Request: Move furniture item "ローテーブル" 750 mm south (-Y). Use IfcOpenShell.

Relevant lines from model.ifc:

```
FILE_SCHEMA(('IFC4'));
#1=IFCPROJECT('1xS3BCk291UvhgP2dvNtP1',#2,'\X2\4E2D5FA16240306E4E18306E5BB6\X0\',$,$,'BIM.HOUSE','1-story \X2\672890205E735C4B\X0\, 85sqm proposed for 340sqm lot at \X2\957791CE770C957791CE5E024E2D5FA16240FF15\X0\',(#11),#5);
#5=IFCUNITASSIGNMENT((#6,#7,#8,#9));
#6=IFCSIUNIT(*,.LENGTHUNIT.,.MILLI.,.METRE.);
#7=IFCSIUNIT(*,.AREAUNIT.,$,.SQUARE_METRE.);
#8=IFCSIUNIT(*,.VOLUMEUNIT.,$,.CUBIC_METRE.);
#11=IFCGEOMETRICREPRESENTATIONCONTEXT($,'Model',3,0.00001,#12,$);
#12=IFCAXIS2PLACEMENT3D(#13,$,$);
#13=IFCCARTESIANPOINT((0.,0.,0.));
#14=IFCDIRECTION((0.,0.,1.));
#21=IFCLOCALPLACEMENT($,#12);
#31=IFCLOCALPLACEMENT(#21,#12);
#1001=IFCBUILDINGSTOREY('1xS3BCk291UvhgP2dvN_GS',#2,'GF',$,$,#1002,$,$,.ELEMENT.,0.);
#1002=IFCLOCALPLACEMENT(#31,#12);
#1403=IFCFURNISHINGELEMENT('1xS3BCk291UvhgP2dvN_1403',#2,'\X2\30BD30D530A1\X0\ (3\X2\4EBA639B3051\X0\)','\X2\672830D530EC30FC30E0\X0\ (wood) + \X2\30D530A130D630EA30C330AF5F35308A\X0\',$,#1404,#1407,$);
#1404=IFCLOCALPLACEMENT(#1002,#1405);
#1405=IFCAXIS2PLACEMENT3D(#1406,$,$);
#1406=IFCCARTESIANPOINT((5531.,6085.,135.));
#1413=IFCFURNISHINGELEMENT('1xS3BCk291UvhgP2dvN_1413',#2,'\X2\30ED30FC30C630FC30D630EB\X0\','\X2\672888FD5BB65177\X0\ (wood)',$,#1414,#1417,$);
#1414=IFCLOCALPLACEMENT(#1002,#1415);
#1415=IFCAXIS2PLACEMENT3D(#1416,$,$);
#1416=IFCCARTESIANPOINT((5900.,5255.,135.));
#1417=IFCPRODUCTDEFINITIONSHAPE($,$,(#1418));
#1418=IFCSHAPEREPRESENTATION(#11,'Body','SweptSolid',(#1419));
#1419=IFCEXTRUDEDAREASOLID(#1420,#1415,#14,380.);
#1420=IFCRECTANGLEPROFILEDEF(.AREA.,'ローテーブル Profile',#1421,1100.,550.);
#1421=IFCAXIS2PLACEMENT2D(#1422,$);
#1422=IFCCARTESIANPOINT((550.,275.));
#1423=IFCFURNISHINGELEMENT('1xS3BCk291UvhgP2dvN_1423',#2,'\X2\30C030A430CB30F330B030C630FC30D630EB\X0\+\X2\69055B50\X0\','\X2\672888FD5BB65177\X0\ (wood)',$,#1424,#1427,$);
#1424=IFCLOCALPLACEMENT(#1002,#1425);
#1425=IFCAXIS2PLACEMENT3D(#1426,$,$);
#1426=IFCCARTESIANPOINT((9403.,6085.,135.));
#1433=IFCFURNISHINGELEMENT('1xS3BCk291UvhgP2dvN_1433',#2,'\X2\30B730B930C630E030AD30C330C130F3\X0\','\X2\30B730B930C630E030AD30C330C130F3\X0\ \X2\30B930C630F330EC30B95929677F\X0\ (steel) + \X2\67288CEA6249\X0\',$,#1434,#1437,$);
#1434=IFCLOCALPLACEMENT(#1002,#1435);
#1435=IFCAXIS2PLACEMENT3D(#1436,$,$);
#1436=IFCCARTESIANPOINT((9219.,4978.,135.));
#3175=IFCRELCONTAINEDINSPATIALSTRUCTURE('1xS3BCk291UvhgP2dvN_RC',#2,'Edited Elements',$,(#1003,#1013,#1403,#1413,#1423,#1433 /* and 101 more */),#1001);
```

```python
import ifcopenshell
import ifcopenshell.api.geometry
import ifcopenshell.util.placement
import ifcopenshell.util.unit

model = ifcopenshell.open("model.ifc")
unit_scale = ifcopenshell.util.unit.calculate_unit_scale(model)

item = model.by_guid("1xS3BCk291UvhgP2dvN_1413")
matrix = ifcopenshell.util.placement.get_local_placement(item.ObjectPlacement)
matrix[1, 3] -= 0.75 / unit_scale
ifcopenshell.api.geometry.edit_object_placement(model, product=item, matrix=matrix, is_si=False)

print(ifcopenshell.util.placement.get_local_placement(item.ObjectPlacement).round(3) + 0.0)

model.write("model_v2.ifc")
```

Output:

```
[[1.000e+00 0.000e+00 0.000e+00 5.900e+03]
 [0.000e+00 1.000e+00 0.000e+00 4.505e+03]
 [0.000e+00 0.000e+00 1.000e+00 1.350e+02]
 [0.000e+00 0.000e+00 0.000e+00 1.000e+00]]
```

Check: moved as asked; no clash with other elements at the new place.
